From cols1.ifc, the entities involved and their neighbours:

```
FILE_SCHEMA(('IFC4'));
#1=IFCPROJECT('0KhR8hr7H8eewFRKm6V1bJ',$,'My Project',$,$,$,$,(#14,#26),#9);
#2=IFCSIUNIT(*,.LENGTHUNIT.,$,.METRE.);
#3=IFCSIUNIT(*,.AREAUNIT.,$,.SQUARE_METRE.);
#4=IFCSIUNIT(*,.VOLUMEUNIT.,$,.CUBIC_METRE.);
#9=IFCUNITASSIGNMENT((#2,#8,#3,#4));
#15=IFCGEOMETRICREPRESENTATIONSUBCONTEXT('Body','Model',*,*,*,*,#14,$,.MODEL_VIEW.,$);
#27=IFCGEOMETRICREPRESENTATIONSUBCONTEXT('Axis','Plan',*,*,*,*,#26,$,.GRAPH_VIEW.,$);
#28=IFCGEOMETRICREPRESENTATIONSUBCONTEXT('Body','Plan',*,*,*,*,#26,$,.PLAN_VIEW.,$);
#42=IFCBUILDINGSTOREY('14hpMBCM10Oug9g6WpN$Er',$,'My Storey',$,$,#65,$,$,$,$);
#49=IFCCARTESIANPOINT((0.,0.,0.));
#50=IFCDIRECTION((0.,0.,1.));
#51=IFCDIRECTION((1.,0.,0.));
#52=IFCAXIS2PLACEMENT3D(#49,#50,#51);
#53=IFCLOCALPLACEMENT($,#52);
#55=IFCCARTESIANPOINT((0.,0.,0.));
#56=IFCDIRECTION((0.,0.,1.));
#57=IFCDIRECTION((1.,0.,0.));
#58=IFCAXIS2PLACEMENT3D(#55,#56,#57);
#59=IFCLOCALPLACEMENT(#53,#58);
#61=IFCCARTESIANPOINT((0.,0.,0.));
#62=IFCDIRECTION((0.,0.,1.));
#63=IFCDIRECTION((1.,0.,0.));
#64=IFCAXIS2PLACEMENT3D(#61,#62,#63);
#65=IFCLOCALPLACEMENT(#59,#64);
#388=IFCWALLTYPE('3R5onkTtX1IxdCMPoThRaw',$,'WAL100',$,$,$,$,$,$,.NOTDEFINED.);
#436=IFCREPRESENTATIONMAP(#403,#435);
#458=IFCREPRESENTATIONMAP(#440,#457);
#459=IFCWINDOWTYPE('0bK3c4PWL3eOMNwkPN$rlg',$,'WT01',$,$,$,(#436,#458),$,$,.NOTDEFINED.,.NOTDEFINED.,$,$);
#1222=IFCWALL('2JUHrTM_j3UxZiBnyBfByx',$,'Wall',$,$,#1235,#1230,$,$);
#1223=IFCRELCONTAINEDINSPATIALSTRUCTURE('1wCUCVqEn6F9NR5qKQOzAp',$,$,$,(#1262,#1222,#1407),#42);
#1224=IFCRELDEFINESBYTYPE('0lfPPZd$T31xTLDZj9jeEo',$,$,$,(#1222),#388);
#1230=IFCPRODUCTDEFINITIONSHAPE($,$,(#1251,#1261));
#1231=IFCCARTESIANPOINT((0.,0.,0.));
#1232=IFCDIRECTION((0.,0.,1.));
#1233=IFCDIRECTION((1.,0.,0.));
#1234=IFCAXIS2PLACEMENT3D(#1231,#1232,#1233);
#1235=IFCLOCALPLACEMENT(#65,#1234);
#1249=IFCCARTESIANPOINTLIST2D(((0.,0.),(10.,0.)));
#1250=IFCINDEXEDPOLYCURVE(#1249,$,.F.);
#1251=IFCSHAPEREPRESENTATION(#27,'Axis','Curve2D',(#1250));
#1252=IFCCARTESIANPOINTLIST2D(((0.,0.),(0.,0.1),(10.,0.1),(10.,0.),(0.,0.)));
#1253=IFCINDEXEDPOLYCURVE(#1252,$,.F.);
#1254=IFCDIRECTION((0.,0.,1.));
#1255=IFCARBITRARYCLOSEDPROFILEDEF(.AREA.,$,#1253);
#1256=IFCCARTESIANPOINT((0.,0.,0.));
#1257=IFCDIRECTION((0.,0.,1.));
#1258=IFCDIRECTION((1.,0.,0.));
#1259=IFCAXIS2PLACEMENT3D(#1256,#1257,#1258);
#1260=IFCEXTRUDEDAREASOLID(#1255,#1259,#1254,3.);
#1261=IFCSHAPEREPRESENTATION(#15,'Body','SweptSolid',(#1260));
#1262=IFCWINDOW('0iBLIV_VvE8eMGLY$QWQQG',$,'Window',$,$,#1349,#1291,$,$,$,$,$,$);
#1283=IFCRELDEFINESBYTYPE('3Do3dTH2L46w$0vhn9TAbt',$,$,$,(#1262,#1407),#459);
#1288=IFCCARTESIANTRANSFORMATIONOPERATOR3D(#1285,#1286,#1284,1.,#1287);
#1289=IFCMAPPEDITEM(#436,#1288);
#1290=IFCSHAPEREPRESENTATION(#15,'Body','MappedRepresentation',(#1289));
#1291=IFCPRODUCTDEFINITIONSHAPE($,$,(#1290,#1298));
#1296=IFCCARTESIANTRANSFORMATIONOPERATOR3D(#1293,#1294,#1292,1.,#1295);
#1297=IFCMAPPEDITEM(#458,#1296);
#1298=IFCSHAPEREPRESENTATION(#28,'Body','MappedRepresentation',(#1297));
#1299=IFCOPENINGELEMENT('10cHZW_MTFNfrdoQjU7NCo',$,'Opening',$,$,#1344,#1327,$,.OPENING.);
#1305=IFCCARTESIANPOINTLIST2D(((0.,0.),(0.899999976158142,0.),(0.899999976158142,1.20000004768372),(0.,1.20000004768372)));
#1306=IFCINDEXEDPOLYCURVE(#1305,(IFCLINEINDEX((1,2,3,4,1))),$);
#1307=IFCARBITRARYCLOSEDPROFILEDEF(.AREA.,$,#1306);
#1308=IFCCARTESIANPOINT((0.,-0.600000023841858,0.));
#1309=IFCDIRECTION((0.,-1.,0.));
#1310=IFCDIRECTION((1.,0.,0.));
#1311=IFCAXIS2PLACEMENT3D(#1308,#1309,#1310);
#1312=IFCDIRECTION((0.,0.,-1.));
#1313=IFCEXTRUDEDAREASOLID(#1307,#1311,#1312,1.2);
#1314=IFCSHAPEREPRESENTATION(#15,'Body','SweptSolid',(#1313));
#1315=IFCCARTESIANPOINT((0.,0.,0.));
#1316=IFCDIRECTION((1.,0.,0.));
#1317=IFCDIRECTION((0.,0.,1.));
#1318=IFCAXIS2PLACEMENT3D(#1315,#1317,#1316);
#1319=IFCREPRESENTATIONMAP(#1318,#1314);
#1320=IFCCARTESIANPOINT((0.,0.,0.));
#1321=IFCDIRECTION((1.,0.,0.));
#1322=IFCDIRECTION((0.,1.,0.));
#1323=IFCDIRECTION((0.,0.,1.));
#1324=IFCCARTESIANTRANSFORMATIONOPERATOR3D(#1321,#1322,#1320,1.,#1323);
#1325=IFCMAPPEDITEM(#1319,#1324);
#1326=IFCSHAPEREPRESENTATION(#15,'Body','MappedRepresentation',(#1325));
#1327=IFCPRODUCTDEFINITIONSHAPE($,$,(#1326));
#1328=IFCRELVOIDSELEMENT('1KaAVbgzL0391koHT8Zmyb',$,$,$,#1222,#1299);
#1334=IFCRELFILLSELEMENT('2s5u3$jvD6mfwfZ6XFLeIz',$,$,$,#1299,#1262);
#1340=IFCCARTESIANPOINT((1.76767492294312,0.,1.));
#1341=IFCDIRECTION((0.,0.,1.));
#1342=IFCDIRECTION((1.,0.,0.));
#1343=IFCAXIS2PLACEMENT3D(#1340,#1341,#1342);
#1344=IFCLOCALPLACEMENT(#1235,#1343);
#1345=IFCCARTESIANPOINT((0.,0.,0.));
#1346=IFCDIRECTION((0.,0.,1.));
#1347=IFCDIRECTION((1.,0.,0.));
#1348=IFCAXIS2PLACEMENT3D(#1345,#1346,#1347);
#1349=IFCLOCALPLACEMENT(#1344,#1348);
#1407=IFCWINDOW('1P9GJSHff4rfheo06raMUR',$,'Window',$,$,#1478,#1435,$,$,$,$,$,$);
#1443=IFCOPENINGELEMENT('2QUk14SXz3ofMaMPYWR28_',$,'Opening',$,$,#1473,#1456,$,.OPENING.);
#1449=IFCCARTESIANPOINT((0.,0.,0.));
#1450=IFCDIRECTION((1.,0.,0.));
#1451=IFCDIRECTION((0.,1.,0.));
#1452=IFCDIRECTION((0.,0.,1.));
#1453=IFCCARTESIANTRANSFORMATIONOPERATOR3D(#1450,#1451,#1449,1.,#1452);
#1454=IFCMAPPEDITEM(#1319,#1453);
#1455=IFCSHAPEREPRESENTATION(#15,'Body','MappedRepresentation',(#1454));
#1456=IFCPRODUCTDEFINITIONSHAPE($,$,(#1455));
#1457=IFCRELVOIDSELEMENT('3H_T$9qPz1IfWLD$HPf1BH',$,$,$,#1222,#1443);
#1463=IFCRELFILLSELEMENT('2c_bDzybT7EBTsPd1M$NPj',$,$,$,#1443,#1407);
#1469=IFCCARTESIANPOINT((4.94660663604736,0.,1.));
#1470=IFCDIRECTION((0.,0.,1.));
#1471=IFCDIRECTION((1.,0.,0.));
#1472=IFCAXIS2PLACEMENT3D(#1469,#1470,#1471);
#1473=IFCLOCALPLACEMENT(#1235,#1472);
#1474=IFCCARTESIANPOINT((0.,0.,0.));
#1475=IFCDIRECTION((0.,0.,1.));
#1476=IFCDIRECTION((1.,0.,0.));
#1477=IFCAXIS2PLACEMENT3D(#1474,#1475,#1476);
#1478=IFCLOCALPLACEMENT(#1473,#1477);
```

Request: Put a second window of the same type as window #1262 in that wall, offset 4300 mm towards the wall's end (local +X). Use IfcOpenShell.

```python
import ifcopenshell
import ifcopenshell.api.feature
import ifcopenshell.api.geometry
import ifcopenshell.api.root
import ifcopenshell.geom
import ifcopenshell.util.element
import ifcopenshell.util.placement
import ifcopenshell.util.shape
import ifcopenshell.util.unit

model = ifcopenshell.open("cols1.ifc")
unit_scale = ifcopenshell.util.unit.calculate_unit_scale(model)
settings = ifcopenshell.geom.settings()


def volume(element):
    """Net volume in cubic metres, openings subtracted."""
    shape = ifcopenshell.geom.create_shape(settings, element)
    return ifcopenshell.util.shape.get_volume(shape.geometry)


window = model.by_id(1262)
opening = window.FillsVoids[0].RelatingOpeningElement
wall = opening.VoidsElements[0].RelatingBuildingElement
before = volume(wall)
shift = ifcopenshell.util.placement.get_local_placement(wall.ObjectPlacement)[:3, 0] * 4.3 / unit_scale

# copy_class copies the void relationship, type, container and properties, but no geometry.
new_opening = ifcopenshell.api.root.copy_class(model, product=opening)
new_opening.Representation = ifcopenshell.util.element.copy_deep(
    model, opening.Representation, exclude=["IfcGeometricRepresentationContext", "IfcRepresentationMap"]
)
new_window = ifcopenshell.api.root.copy_class(model, product=window)
new_window.Representation = ifcopenshell.util.element.copy_deep(
    model, window.Representation, exclude=["IfcGeometricRepresentationContext", "IfcRepresentationMap"]
)
ifcopenshell.api.feature.add_filling(model, opening=new_opening, element=new_window)

for old, new in ((opening, new_opening), (window, new_window)):
    matrix = ifcopenshell.util.placement.get_local_placement(old.ObjectPlacement)
    matrix[:3, 3] += shift
    ifcopenshell.api.geometry.edit_object_placement(model, product=new, matrix=matrix, is_si=False)

after = volume(wall)

print(f"wall volume {before:.3f} -> {after:.3f} m3")

model.write("cols1_rev.ifc")
```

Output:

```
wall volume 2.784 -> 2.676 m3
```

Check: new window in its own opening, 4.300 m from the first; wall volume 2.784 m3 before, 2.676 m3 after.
